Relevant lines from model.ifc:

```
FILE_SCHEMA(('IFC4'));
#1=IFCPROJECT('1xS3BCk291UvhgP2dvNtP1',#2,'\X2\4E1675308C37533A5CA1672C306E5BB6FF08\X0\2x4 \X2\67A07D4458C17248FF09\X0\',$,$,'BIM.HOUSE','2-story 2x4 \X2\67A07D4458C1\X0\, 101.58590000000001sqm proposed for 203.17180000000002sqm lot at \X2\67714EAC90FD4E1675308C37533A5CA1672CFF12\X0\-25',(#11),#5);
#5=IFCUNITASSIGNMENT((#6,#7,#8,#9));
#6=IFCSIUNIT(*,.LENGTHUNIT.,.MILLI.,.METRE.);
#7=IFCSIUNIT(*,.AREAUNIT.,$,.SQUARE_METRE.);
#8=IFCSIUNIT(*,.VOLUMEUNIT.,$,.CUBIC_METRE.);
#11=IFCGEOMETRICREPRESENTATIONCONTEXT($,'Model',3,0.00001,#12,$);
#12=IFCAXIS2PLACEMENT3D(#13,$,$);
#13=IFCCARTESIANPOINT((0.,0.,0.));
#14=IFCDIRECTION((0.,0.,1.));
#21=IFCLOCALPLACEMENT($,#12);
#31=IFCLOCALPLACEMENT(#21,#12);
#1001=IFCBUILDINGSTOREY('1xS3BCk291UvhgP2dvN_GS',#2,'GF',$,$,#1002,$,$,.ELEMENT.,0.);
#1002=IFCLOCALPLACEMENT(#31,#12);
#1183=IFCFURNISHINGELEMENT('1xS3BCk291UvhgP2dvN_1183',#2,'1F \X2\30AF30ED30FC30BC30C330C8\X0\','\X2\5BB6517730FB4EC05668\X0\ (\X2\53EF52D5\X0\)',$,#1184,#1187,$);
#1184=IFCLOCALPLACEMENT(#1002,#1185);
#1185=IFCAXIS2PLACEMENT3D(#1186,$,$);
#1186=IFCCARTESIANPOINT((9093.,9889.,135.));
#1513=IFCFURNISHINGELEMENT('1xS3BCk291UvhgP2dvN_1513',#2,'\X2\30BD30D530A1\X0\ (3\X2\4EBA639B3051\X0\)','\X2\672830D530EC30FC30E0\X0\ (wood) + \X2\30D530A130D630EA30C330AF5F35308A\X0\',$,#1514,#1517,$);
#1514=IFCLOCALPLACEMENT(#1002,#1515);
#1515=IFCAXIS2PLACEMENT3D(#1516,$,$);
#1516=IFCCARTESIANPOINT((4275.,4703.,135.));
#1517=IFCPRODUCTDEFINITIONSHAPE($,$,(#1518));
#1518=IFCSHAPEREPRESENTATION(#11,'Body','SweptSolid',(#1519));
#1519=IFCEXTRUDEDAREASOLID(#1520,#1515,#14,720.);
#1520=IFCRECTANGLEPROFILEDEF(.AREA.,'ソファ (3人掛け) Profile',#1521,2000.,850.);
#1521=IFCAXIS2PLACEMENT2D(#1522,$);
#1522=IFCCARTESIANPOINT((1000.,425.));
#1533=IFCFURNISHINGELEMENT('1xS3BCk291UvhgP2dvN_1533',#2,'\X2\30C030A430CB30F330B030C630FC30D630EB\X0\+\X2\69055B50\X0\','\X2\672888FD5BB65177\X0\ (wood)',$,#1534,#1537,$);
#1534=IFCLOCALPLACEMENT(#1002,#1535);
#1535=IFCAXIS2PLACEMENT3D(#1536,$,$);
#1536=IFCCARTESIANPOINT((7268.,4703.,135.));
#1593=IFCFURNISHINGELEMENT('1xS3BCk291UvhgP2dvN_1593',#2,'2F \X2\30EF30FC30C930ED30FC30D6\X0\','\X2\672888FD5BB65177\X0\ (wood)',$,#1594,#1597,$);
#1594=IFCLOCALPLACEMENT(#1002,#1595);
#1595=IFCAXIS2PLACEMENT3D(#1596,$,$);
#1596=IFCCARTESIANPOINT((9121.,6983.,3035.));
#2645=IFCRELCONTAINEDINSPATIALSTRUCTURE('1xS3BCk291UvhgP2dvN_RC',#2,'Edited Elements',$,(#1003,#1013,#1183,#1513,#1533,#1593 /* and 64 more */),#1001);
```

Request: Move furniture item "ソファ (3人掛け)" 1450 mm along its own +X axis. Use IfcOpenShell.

```python
import ifcopenshell
import ifcopenshell.api.geometry
import ifcopenshell.util.placement

model = ifcopenshell.open("model.ifc")

item = model.by_guid("1xS3BCk291UvhgP2dvN_1513")
matrix = ifcopenshell.util.placement.get_local_placement(item.ObjectPlacement)
matrix[:3, 3] += matrix[:3, 0] * 1450.0
ifcopenshell.api.geometry.edit_object_placement(model, product=item, matrix=matrix, is_si=False)

print(ifcopenshell.util.placement.get_local_placement(item.ObjectPlacement).round(3) + 0.0)

model.write("model-out.ifc")
```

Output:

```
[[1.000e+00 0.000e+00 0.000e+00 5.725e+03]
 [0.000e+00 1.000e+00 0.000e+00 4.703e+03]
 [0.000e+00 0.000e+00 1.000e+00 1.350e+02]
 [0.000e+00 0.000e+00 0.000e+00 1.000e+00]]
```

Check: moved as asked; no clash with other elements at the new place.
